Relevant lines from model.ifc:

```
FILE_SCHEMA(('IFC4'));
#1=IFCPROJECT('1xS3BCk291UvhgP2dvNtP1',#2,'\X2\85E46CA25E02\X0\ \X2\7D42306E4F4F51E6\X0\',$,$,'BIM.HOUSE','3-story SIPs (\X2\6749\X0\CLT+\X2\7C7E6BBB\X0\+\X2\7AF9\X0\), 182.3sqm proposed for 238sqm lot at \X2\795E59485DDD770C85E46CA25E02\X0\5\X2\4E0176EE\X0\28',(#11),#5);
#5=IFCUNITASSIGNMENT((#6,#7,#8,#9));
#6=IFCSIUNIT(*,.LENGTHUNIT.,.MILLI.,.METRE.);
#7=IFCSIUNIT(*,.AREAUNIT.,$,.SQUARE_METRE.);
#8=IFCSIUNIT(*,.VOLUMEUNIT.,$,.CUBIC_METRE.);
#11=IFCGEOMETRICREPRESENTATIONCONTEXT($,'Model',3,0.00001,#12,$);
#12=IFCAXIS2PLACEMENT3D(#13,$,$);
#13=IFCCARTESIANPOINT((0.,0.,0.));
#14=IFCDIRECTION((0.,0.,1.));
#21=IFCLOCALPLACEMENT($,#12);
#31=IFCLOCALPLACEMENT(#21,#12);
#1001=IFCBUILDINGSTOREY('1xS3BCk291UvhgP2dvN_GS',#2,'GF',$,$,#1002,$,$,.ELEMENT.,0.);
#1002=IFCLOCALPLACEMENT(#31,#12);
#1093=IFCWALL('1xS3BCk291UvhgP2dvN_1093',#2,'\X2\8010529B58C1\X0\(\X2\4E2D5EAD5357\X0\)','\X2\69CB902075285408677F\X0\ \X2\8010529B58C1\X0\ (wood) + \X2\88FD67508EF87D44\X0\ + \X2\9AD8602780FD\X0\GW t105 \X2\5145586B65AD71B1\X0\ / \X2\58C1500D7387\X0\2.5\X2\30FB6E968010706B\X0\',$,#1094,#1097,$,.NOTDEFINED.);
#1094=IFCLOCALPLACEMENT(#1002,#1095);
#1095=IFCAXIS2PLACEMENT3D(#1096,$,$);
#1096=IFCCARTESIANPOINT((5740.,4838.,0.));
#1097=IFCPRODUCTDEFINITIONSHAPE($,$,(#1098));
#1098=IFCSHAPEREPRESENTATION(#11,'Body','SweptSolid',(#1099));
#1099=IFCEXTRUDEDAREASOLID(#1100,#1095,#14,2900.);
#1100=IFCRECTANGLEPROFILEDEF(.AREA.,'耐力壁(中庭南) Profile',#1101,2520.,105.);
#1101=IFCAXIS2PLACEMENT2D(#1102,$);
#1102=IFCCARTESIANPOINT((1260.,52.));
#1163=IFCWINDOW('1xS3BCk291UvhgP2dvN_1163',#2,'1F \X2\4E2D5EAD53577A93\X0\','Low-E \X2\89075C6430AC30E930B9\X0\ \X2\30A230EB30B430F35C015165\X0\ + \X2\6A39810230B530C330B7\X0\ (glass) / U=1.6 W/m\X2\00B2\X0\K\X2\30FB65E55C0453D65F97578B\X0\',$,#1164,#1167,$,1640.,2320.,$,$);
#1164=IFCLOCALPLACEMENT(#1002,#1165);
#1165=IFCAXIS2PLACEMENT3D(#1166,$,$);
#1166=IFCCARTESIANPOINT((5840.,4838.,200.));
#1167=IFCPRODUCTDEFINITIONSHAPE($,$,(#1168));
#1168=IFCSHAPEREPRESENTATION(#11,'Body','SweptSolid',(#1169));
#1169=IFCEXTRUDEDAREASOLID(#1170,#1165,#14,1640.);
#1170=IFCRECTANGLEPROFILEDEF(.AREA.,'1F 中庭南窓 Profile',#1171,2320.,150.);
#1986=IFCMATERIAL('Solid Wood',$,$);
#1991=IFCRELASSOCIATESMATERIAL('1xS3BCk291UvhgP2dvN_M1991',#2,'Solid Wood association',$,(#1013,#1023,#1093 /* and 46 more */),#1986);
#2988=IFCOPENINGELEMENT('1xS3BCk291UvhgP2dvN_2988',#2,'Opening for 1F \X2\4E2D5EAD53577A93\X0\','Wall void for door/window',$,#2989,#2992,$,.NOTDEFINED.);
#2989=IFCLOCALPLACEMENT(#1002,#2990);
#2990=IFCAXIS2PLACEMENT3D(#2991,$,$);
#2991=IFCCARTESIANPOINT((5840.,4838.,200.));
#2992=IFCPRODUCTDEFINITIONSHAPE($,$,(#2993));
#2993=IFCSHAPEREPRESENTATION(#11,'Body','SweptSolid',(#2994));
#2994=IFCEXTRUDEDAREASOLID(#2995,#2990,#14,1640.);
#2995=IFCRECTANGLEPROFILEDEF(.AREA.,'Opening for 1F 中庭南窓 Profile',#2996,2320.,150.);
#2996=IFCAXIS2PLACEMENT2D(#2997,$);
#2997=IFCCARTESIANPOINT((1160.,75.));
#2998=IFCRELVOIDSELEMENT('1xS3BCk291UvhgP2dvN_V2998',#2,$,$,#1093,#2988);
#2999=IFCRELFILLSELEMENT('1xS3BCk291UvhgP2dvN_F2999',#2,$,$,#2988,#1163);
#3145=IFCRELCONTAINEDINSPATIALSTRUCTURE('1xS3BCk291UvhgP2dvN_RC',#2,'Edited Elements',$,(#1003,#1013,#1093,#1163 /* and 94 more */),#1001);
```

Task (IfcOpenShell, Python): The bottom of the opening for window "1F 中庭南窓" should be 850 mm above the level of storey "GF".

```python
import numpy as np
import ifcopenshell
import ifcopenshell.api.geometry
import ifcopenshell.geom
import ifcopenshell.util.element
import ifcopenshell.util.placement
import ifcopenshell.util.shape
import ifcopenshell.util.unit

model = ifcopenshell.open("model.ifc")
unit_scale = ifcopenshell.util.unit.calculate_unit_scale(model)

window = model.by_id(1163)
opening = window.FillsVoids[0].RelatingOpeningElement
storey = ifcopenshell.util.element.get_container(window, ifc_class="IfcBuildingStorey")
level = ifcopenshell.util.placement.get_local_placement(storey.ObjectPlacement)[2, 3]

# The opening's origin need not be at the sill, so measure its lowest point.
shape = ifcopenshell.geom.create_shape(ifcopenshell.geom.settings(), opening)
bottom = ifcopenshell.util.shape.get_shape_bottom_elevation(shape, shape.geometry) / unit_scale
dz = level + 850.0 - bottom

shift = np.array([0.0, 0.0, dz])
# The window is not placed relative to its opening, so move both.
for product in (opening, window):
    matrix = ifcopenshell.util.placement.get_local_placement(product.ObjectPlacement)
    matrix[:3, 3] += shift
    ifcopenshell.api.geometry.edit_object_placement(model, product=product, matrix=matrix, is_si=False)

print(f"moved by {dz * unit_scale:+.3f} m")

model.write("model_rev.ifc")
```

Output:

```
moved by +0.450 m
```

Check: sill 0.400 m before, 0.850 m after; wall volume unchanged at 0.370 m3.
